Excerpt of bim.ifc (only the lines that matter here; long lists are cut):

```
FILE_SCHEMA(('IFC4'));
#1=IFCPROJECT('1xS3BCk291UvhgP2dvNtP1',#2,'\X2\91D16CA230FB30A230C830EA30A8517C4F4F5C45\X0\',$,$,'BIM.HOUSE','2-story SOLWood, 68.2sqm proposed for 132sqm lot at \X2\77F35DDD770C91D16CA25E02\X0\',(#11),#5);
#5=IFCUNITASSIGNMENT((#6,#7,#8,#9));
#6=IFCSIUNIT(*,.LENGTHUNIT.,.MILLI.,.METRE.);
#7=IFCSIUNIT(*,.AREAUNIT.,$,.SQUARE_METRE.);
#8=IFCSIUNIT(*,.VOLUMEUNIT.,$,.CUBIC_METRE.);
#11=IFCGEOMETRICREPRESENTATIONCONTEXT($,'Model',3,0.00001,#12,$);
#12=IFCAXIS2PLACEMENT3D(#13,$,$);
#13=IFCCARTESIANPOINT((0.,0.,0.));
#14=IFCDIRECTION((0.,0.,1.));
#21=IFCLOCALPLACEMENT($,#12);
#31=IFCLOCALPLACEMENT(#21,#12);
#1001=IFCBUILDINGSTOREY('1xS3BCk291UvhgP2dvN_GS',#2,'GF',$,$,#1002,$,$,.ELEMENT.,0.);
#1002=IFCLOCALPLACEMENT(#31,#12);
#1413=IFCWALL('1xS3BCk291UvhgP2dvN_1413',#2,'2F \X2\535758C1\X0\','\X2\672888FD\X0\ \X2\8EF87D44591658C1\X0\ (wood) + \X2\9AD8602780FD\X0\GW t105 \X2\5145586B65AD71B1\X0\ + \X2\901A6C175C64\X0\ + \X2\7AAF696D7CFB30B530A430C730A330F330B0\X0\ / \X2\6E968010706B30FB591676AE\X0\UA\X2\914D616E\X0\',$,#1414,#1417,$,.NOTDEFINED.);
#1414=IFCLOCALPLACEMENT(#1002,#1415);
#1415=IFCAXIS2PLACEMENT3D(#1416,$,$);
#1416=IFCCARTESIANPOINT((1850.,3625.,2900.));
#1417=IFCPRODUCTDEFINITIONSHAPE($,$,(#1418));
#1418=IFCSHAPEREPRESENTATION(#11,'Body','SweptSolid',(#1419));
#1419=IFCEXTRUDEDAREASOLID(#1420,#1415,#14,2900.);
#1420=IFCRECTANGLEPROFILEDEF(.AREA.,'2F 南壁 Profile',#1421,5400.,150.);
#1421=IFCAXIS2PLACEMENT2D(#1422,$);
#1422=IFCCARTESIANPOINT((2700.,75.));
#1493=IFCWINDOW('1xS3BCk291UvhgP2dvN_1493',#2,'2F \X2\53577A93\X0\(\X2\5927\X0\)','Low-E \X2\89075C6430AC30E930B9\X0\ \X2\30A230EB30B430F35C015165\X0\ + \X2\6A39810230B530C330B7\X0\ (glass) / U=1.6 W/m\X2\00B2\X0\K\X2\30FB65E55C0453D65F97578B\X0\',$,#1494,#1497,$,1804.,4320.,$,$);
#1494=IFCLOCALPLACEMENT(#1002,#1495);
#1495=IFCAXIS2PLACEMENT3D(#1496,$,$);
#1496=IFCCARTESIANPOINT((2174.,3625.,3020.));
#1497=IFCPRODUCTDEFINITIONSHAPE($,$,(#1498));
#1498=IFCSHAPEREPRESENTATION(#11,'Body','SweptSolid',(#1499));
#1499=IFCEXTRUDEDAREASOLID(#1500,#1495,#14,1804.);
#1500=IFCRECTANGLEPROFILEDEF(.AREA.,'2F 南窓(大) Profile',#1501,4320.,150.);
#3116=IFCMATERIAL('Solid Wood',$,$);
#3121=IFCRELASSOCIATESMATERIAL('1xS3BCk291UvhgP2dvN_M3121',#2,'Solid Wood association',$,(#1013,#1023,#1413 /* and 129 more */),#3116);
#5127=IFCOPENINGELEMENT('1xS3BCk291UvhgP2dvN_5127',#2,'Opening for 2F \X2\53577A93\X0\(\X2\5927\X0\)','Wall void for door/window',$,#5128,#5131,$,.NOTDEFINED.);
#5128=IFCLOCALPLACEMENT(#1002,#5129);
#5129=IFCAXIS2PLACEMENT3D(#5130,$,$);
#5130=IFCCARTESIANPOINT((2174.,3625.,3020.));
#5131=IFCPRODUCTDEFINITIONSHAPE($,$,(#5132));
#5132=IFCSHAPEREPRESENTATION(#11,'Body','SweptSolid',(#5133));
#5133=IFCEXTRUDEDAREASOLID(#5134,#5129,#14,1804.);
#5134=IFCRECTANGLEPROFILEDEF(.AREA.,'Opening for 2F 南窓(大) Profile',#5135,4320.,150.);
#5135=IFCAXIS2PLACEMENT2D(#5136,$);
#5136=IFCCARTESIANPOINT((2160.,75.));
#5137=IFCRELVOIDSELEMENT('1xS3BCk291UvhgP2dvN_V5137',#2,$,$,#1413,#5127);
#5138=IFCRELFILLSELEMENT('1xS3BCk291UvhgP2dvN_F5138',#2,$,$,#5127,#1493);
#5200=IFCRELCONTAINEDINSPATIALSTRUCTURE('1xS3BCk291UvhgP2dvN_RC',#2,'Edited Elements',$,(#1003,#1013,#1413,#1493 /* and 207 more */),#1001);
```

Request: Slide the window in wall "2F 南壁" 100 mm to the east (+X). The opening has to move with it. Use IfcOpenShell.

```python
import ifcopenshell
import ifcopenshell.api.geometry
import ifcopenshell.util.placement
import ifcopenshell.util.unit

model = ifcopenshell.open("bim.ifc")
unit_scale = ifcopenshell.util.unit.calculate_unit_scale(model)

window = model.by_guid("1xS3BCk291UvhgP2dvN_1493")
opening = window.FillsVoids[0].RelatingOpeningElement
wall = opening.VoidsElements[0].RelatingBuildingElement

wall_matrix = ifcopenshell.util.placement.get_local_placement(wall.ObjectPlacement)
shift = wall_matrix[:3, 0] * 0.1 / unit_scale
before = ifcopenshell.util.placement.get_local_placement(window.ObjectPlacement)[:3, 3].copy()

# The window is not placed relative to its opening, so move both.
for product in (opening, window):
    matrix = ifcopenshell.util.placement.get_local_placement(product.ObjectPlacement)
    matrix[:3, 3] += shift
    ifcopenshell.api.geometry.edit_object_placement(model, product=product, matrix=matrix, is_si=False)

after = ifcopenshell.util.placement.get_local_placement(window.ObjectPlacement)[:3, 3]
print("window moved by", (after - before).round(3) + 0.0)

model.write("bim-out.ifc")
```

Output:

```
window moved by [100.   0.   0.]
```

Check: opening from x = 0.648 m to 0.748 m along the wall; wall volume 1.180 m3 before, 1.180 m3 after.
